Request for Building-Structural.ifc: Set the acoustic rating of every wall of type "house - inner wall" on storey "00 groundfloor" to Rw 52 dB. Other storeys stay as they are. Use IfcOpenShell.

First a look at what the model holds.

```python
import ifcopenshell
import ifcopenshell.util.element

model = ifcopenshell.open("Building-Structural.ifc")
print(model.schema)
storey = next(s for s in model.by_type("IfcBuildingStorey") if s.Name == "00 groundfloor")
walls = [e for e in ifcopenshell.util.element.get_decomposition(storey) if e.is_a("IfcWall")]
seen = {}
for e in walls:
    element_type = ifcopenshell.util.element.get_type(e)
    key = (element_type.Name if element_type != e and element_type else None, ifcopenshell.util.element.get_pset(e, "Pset_WallCommon", "AcousticRating"))
    seen[key] = seen.get(key, 0) + 1
for (name, value), count in sorted(seen.items(), key=str):
    print(count, "x", name, "|", value)
```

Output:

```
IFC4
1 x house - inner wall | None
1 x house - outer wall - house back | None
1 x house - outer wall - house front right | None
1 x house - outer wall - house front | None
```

```python
import ifcopenshell
import ifcopenshell.api.pset
import ifcopenshell.util.element

model = ifcopenshell.open("Building-Structural.ifc")

storey = next(s for s in model.by_type("IfcBuildingStorey") if s.Name == "00 groundfloor")
walls = [e for e in ifcopenshell.util.element.get_decomposition(storey) if e.is_a("IfcWall")]

count = 0
for e in walls:
    element_type = ifcopenshell.util.element.get_type(e)
    if element_type in (None, e) or element_type.Name != "house - inner wall":
        continue
    # add_pset returns the element's existing set when there is one.
    pset = ifcopenshell.api.pset.add_pset(model, product=e, name="Pset_WallCommon")
    ifcopenshell.api.pset.edit_pset(model, pset=pset, properties={"AcousticRating": "Rw 52 dB"})
    count += 1

print(count, "walls updated")

model.write("Building-Structural-out.ifc")
```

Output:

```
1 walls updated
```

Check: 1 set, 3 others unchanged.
